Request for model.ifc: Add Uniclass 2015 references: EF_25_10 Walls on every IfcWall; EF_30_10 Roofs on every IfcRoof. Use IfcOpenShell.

First a look at what the model holds.

```python
import ifcopenshell

model = ifcopenshell.open("model.ifc")
print(model.schema)
print("classifications:", [c.Name for c in model.by_type("IfcClassification")])
for ifc_class in ("IfcDoor", "IfcRoof", "IfcStair", "IfcWall", "IfcWindow"):
    print(ifc_class, len(model.by_type(ifc_class)))
```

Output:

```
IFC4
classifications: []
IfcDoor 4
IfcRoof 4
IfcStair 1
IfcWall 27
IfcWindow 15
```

```python
import ifcopenshell
import ifcopenshell.api.classification

model = ifcopenshell.open("model.ifc")

system = ifcopenshell.api.classification.add_classification(model, classification="Uniclass 2015")

codes = {
    "IfcWall": ("EF_25_10", "Walls"),
    "IfcRoof": ("EF_30_10", "Roofs"),
}
for ifc_class, (code, name) in codes.items():
    products = model.by_type(ifc_class)
    ifcopenshell.api.classification.add_reference(
        model, products=products, classification=system, identification=code, name=name
    )
    print(code, len(products))

model.write("model-out.ifc")
```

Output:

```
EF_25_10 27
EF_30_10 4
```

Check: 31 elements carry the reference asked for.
